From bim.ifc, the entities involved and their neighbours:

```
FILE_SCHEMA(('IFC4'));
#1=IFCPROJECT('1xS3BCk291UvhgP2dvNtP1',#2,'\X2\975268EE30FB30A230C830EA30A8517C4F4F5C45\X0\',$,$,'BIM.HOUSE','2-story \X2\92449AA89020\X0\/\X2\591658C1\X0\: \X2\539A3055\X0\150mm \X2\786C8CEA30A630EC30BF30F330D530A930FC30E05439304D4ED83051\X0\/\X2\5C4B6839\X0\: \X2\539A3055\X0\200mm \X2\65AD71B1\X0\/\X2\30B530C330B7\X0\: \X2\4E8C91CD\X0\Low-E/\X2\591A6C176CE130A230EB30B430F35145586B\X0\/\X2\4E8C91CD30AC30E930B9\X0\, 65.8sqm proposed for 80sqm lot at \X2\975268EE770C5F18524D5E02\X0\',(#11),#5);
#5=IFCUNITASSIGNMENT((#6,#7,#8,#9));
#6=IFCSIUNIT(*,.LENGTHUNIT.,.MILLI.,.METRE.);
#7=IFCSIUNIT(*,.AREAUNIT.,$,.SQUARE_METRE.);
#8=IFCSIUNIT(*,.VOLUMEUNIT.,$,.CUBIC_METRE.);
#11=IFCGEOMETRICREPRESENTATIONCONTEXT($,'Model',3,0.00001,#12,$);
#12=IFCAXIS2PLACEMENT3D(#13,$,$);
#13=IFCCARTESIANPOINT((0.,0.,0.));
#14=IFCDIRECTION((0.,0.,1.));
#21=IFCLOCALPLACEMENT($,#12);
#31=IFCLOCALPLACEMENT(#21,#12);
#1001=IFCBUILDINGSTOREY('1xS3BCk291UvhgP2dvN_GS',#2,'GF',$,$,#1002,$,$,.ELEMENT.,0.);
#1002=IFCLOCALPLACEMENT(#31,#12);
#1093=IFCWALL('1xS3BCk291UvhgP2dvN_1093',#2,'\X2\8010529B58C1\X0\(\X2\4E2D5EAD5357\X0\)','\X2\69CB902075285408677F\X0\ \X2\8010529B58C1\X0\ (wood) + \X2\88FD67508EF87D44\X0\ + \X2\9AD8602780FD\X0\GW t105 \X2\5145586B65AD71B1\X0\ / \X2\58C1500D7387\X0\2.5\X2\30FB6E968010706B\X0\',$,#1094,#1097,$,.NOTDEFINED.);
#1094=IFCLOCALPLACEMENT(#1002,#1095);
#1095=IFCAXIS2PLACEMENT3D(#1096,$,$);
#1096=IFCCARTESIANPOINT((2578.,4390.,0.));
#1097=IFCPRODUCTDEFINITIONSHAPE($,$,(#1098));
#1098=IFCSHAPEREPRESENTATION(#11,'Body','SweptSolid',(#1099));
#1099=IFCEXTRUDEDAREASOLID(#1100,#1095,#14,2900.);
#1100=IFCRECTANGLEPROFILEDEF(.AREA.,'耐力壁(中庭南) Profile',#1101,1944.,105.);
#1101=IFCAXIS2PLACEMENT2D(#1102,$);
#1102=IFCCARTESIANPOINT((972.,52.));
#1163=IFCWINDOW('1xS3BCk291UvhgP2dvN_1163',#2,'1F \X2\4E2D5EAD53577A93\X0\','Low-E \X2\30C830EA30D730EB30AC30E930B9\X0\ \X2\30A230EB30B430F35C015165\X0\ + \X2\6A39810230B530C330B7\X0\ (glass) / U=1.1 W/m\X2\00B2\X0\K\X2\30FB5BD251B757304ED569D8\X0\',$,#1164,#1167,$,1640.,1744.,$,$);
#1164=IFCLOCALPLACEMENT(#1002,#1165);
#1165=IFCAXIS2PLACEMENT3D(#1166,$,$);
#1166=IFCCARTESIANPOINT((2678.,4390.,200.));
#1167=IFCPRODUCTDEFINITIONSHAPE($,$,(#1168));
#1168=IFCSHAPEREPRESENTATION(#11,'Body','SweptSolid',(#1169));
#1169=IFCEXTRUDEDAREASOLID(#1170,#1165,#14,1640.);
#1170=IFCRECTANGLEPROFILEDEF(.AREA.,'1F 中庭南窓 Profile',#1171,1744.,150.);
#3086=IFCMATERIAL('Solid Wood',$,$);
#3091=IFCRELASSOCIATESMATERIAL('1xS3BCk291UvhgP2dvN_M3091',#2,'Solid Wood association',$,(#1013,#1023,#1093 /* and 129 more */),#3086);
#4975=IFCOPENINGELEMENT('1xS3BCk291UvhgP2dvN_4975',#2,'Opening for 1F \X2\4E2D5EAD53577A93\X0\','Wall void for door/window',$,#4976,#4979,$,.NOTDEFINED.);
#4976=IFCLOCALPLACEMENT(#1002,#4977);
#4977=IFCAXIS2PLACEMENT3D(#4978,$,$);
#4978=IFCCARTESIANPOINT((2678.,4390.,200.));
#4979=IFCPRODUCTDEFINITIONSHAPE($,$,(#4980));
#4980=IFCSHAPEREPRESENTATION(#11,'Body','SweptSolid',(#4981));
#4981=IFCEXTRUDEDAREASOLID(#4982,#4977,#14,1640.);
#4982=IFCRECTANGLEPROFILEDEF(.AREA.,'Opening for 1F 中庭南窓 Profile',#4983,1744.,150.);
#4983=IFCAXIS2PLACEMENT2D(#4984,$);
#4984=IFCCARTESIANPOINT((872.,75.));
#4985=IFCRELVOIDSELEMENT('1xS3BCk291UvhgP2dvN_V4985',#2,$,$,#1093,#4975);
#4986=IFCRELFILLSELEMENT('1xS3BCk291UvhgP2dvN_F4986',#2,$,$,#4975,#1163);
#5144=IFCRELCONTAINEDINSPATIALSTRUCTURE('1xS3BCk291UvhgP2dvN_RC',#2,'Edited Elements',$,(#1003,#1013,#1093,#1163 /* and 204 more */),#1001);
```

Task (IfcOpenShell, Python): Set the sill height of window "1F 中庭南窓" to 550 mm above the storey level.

```python
import numpy as np
import ifcopenshell
import ifcopenshell.api.geometry
import ifcopenshell.geom
import ifcopenshell.util.element
import ifcopenshell.util.placement
import ifcopenshell.util.shape
import ifcopenshell.util.unit

model = ifcopenshell.open("bim.ifc")
unit_scale = ifcopenshell.util.unit.calculate_unit_scale(model)

window = model.by_guid("1xS3BCk291UvhgP2dvN_1163")
opening = window.FillsVoids[0].RelatingOpeningElement
storey = ifcopenshell.util.element.get_container(window, ifc_class="IfcBuildingStorey")
level = ifcopenshell.util.placement.get_local_placement(storey.ObjectPlacement)[2, 3]

# The opening's origin need not be at the sill, so measure its lowest point.
shape = ifcopenshell.geom.create_shape(ifcopenshell.geom.settings(), opening)
bottom = ifcopenshell.util.shape.get_shape_bottom_elevation(shape, shape.geometry) / unit_scale
dz = level + 550.0 - bottom

shift = np.array([0.0, 0.0, dz])
# The window is not placed relative to its opening, so move both.
for product in (opening, window):
    matrix = ifcopenshell.util.placement.get_local_placement(product.ObjectPlacement)
    matrix[:3, 3] += shift
    ifcopenshell.api.geometry.edit_object_placement(model, product=product, matrix=matrix, is_si=False)

print(f"moved by {dz * unit_scale:+.3f} m")

model.write("bim_rev.ifc")
```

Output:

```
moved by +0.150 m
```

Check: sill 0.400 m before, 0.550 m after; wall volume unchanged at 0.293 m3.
